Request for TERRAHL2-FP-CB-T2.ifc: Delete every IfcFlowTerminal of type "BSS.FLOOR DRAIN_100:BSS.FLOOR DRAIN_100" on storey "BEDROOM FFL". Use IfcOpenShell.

First a look at what the model holds.

```python
import ifcopenshell
import ifcopenshell.util.element

model = ifcopenshell.open("TERRAHL2-FP-CB-T2.ifc")
print(model.schema)
storey = next(s for s in model.by_type("IfcBuildingStorey") if s.Name == "BEDROOM FFL")
terminals = [e for e in ifcopenshell.util.element.get_decomposition(storey) if e.is_a("IfcFlowTerminal")]
seen = {}
for e in terminals:
    element_type = ifcopenshell.util.element.get_type(e)
    name = element_type.Name if element_type not in (None, e) else None
    seen[name] = seen.get(name, 0) + 1
for name, count in sorted(seen.items(), key=str):
    print(count, "x", name)
```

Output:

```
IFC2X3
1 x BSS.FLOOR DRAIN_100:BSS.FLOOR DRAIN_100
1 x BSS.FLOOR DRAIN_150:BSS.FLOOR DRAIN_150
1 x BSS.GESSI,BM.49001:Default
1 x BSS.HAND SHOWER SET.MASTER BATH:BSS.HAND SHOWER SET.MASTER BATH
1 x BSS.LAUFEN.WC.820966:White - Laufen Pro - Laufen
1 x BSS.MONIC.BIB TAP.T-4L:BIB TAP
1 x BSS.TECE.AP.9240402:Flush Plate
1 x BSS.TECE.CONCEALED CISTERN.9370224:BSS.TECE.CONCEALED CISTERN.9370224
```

```python
import ifcopenshell
import ifcopenshell.api.root
import ifcopenshell.util.element

model = ifcopenshell.open("TERRAHL2-FP-CB-T2.ifc")

storey = next(s for s in model.by_type("IfcBuildingStorey") if s.Name == "BEDROOM FFL")
terminals = [e for e in ifcopenshell.util.element.get_decomposition(storey) if e.is_a("IfcFlowTerminal")]
targets = [e for e in terminals if (t := ifcopenshell.util.element.get_type(e)) not in (None, e) and t.Name == "BSS.FLOOR DRAIN_100:BSS.FLOOR DRAIN_100"]

for e in targets:
    ifcopenshell.api.root.remove_product(model, product=e)
print(len(targets), "removed")

model.write("TERRAHL2-FP-CB-T2_v2.ifc")
```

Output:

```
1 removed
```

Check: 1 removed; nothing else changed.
